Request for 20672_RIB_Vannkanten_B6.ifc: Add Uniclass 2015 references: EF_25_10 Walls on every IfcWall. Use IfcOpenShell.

First a look at what the model holds.

```python
import ifcopenshell

model = ifcopenshell.open("20672_RIB_Vannkanten_B6.ifc")
print(model.schema)
print("classifications:", [c.Name for c in model.by_type("IfcClassification")])
for ifc_class in ("IfcDoor", "IfcRoof", "IfcStair", "IfcWall", "IfcWindow"):
    print(ifc_class, len(model.by_type(ifc_class)))
```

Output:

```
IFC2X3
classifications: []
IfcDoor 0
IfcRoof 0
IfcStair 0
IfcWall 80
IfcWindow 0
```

```python
import ifcopenshell
import ifcopenshell.api.classification

model = ifcopenshell.open("20672_RIB_Vannkanten_B6.ifc")

# IFC2X3 requires Source and Edition and has no link from the project to the system.
system = model.create_entity("IfcClassification", Source="NBS", Edition="2015", Name="Uniclass 2015")

codes = {
    "IfcWall": ("EF_25_10", "Walls"),
}
for ifc_class, (code, name) in codes.items():
    products = model.by_type(ifc_class)
    ifcopenshell.api.classification.add_reference(
        model, products=products, classification=system, identification=code, name=name
    )
    print(code, len(products))

model.write("20672_RIB_Vannkanten_B6-out.ifc")
```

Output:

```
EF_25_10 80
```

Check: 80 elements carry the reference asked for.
